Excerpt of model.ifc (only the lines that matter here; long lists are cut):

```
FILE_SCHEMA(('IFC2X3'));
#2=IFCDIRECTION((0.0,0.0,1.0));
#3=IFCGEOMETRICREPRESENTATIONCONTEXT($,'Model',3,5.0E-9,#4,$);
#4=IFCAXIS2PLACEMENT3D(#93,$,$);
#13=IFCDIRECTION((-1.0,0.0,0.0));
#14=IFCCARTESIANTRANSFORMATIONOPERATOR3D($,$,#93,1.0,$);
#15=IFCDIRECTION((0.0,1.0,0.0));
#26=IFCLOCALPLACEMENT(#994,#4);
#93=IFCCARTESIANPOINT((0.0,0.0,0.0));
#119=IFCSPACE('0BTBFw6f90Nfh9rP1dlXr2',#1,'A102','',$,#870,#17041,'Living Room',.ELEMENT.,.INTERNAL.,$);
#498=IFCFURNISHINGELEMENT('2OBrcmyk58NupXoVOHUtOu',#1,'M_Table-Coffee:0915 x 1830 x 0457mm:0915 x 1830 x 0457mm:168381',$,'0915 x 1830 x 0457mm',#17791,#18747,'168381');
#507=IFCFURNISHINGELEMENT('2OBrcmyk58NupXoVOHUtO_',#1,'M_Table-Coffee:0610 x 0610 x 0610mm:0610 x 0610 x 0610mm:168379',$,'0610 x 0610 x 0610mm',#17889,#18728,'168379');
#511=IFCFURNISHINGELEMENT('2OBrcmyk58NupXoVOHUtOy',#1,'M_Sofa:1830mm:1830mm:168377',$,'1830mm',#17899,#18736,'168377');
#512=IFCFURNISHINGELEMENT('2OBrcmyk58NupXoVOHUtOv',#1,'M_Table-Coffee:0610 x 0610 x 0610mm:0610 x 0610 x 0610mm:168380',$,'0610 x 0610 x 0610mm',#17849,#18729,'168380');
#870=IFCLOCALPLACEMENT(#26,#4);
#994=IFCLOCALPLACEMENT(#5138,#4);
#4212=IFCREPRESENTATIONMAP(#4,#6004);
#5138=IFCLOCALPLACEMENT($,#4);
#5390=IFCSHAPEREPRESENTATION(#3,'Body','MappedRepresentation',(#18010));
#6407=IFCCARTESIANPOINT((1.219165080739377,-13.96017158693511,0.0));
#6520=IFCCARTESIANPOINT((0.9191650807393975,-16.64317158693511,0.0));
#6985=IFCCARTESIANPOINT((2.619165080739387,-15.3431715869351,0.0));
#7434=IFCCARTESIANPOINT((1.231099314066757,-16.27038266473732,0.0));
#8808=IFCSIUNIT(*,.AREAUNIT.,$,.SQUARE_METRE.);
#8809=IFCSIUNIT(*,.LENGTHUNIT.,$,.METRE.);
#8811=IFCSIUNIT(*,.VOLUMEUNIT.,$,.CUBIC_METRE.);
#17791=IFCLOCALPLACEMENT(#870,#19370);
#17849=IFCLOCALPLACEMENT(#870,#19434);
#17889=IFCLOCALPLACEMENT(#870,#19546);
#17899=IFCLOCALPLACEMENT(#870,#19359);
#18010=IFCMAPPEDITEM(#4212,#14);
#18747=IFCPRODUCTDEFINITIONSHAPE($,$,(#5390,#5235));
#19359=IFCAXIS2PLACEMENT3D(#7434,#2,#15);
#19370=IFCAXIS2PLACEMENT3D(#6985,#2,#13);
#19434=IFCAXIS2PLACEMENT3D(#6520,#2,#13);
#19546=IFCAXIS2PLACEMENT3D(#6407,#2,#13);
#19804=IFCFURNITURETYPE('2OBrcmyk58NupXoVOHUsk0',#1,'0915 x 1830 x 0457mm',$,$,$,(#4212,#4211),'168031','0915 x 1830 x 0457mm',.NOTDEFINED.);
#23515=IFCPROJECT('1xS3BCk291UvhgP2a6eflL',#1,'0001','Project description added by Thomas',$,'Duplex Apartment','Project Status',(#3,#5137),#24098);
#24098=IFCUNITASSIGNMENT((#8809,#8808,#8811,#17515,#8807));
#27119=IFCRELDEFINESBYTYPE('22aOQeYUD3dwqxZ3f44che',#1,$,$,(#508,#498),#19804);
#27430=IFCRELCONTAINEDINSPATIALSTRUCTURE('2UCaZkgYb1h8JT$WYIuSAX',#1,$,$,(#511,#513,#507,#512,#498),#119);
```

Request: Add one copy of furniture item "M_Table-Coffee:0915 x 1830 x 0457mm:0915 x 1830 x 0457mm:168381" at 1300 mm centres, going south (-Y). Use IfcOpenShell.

```python
import numpy as np
import ifcopenshell
import ifcopenshell.api.geometry
import ifcopenshell.api.root
import ifcopenshell.util.element
import ifcopenshell.util.placement

model = ifcopenshell.open("model.ifc")


def reuse_history(source, copy):
    """copy_class also copies each property set's owner history, people and application; keep the originals."""
    for rel in copy.IsDefinedBy:
        if rel.is_a("IfcRelDefinesByProperties") and (history := rel.RelatingPropertyDefinition.OwnerHistory):
            rel.RelatingPropertyDefinition.OwnerHistory = source.OwnerHistory
            ifcopenshell.util.element.remove_deep2(model, history)


source = model.by_id(498)
base = ifcopenshell.util.placement.get_local_placement(source.ObjectPlacement)
step = np.array([0.0, -1.0, 0.0]) * 1.3

for i in range(1, 2):
    copy = ifcopenshell.api.root.copy_class(model, product=source)
    copy.Representation = ifcopenshell.util.element.copy_deep(
        model, source.Representation, exclude=["IfcGeometricRepresentationContext", "IfcRepresentationMap"]
    )
    copy.Name = "M_Table-Coffee:0915 x 1830 x 0457mm:0915 x 1830 x 0457mm"
    copy.Tag = None
    reuse_history(source, copy)
    matrix = base.copy()
    matrix[:3, 3] += i * step
    print("added at", matrix[:3, 3].round(3) + 0.0)
    ifcopenshell.api.geometry.edit_object_placement(model, product=copy, matrix=matrix, is_si=False)

model.write("model_edited.ifc")
```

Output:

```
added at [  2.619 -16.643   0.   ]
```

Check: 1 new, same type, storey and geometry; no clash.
